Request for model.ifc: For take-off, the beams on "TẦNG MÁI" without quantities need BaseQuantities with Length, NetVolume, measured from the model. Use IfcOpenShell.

First a look at what the model holds.

```python
import ifcopenshell
import ifcopenshell.util.element
import ifcopenshell.util.unit

model = ifcopenshell.open("model.ifc")
print(model.schema)
for unit_type in ("LENGTHUNIT", "AREAUNIT", "VOLUMEUNIT"):
    print(unit_type, ifcopenshell.util.unit.calculate_unit_scale(model, unit_type))
storey = next(s for s in model.by_type("IfcBuildingStorey") if s.Name == "TẦNG MÁI")
beams = [e for e in ifcopenshell.util.element.get_decomposition(storey) if e.is_a("IfcBeam")]
for e in sorted(beams, key=lambda e: e.id()):
    print(e.id(), e.is_a(), e.Name, list(ifcopenshell.util.element.get_psets(e, qtos_only=True)), sep=" | ")
```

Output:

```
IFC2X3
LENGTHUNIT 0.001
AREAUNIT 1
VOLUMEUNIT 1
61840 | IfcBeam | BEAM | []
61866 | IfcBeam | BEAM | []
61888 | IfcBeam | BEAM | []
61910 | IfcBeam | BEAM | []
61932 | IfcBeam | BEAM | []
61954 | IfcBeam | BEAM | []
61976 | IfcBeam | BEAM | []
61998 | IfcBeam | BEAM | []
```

```python
import ifcopenshell
import ifcopenshell.api.pset
import ifcopenshell.geom
import ifcopenshell.util.element
import ifcopenshell.util.shape
import ifcopenshell.util.unit

model = ifcopenshell.open("model.ifc")
unit_scale = ifcopenshell.util.unit.calculate_unit_scale(model)
volume_scale = ifcopenshell.util.unit.calculate_unit_scale(model, "VOLUMEUNIT")
settings = ifcopenshell.geom.settings()

storey = next(s for s in model.by_type("IfcBuildingStorey") if s.Name == "TẦNG MÁI")
beams = [e for e in ifcopenshell.util.element.get_decomposition(storey) if e.is_a("IfcBeam")]

for e in sorted(beams, key=lambda e: e.id()):
    if ifcopenshell.util.element.get_psets(e, qtos_only=True, should_inherit=False):
        continue
    # Geometry comes back in metres, in the element's own axes.
    shape = ifcopenshell.geom.create_shape(settings, e)
    values = {
        "Length": ifcopenshell.util.shape.get_max_xyz(shape.geometry) / unit_scale,
        "NetVolume": ifcopenshell.util.shape.get_volume(shape.geometry) / volume_scale,
    }
    qto = ifcopenshell.api.pset.add_qto(model, product=e, name="BaseQuantities")
    ifcopenshell.api.pset.edit_qto(model, qto=qto, properties=values)
    print(e.id(), {k: round(v, 3) for k, v in values.items()})

model.write("model_rev.ifc")
```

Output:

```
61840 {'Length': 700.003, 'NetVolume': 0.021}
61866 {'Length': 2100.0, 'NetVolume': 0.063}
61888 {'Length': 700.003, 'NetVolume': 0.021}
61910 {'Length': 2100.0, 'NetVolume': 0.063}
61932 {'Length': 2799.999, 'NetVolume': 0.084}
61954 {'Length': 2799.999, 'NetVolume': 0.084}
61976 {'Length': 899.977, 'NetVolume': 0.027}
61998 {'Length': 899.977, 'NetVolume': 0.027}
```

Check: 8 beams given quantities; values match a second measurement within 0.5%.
